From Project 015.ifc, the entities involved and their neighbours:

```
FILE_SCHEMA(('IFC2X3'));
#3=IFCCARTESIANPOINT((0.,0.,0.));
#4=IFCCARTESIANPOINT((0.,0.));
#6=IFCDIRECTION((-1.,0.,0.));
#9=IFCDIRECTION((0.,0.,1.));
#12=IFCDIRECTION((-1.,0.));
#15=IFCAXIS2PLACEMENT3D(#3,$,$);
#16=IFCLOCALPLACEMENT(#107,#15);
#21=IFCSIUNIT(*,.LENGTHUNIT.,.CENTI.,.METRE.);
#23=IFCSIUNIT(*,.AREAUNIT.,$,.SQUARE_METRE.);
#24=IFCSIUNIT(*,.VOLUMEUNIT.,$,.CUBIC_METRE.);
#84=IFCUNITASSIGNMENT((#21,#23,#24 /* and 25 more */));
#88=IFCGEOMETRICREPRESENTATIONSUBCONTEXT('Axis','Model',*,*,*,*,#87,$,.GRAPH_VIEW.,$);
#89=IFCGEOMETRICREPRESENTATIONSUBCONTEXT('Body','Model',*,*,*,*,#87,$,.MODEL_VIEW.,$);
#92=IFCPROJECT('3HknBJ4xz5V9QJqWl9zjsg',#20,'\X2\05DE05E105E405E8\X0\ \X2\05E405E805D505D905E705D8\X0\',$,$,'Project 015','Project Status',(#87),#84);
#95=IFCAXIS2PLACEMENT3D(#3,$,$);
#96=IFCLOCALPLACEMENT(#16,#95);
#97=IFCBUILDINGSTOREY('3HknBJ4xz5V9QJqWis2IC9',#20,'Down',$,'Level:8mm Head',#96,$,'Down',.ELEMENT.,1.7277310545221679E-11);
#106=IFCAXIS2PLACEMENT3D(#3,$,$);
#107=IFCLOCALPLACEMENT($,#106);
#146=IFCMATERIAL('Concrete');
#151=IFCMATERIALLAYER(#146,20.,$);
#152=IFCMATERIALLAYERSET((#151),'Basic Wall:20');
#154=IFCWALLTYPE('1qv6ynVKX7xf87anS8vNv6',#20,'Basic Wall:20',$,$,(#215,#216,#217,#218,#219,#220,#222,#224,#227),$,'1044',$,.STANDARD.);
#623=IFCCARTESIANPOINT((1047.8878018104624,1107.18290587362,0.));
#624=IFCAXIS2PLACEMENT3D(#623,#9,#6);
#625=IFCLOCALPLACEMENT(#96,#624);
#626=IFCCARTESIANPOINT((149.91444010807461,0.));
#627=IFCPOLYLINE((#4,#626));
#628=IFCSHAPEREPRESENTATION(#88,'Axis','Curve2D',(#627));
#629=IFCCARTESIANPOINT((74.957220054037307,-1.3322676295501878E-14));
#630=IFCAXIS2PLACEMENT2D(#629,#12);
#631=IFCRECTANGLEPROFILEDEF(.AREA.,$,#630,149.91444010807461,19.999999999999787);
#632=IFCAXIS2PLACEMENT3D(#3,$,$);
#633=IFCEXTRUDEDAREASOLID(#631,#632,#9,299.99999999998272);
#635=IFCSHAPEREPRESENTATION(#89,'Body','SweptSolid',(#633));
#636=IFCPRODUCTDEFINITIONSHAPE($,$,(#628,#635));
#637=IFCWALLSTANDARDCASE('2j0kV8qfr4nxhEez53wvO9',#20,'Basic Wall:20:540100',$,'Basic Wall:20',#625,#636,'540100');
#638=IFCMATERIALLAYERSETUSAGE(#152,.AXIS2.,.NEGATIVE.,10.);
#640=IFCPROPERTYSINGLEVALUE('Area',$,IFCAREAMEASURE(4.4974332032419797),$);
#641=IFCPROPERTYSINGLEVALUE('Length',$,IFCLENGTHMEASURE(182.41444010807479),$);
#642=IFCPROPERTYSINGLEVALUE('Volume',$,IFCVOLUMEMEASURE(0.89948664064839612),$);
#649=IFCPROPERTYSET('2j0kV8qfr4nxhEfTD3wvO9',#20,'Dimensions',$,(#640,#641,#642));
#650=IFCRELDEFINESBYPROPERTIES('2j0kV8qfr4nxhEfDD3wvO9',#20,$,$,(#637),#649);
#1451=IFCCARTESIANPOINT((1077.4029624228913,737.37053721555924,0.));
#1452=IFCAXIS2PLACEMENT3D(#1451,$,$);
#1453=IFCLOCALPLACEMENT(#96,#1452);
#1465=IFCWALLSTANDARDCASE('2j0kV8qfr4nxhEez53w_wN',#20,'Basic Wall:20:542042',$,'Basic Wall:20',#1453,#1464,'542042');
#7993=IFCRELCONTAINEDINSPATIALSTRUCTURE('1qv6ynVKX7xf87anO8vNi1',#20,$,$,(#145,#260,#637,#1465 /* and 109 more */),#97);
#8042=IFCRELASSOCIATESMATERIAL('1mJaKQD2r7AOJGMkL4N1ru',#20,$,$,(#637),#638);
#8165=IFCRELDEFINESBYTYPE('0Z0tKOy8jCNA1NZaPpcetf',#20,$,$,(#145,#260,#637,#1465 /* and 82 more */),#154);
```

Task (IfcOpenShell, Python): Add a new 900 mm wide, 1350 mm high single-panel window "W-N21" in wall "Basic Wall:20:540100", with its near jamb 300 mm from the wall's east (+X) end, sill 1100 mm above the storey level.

```python
import numpy as np
import ifcopenshell
import ifcopenshell.api.feature
import ifcopenshell.api.geometry
import ifcopenshell.api.pset
import ifcopenshell.api.root
import ifcopenshell.api.spatial
import ifcopenshell.api.type
import ifcopenshell.geom
import ifcopenshell.util.element
import ifcopenshell.util.placement
import ifcopenshell.util.representation
import ifcopenshell.util.shape
import ifcopenshell.util.unit

model = ifcopenshell.open("Project 015.ifc")
unit_scale = ifcopenshell.util.unit.calculate_unit_scale(model)
area_scale = ifcopenshell.util.unit.calculate_unit_scale(model, "AREAUNIT")
volume_scale = ifcopenshell.util.unit.calculate_unit_scale(model, "VOLUMEUNIT")
settings = ifcopenshell.geom.settings()


def volume(element):
    """Net volume in cubic metres, openings subtracted."""
    shape = ifcopenshell.geom.create_shape(settings, element)
    return ifcopenshell.util.shape.get_volume(shape.geometry)


wall = model.by_id(637)
storey = ifcopenshell.util.element.get_container(wall, ifc_class="IfcBuildingStorey")
context = ifcopenshell.util.representation.get_context(model, "Model", "Body", "MODEL_VIEW")
before = volume(wall)

width, height, from_end, sill = 0.9, 1.35, 0.3, 1.1  # metres

# The wall runs along its own X axis, and the end named is its -X end.
wall_shape = ifcopenshell.geom.create_shape(settings, wall)
x, y, z = ifcopenshell.util.shape.get_vertices(wall_shape.geometry).T
start = x.min() + from_end
face, thickness = float(y.min()), float(y.max() - y.min())
wall_matrix = ifcopenshell.util.placement.get_local_placement(wall.ObjectPlacement)
level = ifcopenshell.util.placement.get_local_placement(storey.ObjectPlacement)[2, 3]


def in_wall(x, y):
    """Placement at x, y metres in the wall's axes, at sill height."""
    matrix = wall_matrix.copy()
    matrix[:, 3] = wall_matrix @ np.array([x / unit_scale, y / unit_scale, 0.0, 1.0])
    matrix[2, 3] = level + sill / unit_scale
    return matrix


# Opening: a box that overshoots both wall faces by 50 mm.
opening = ifcopenshell.api.root.create_entity(model, ifc_class="IfcOpeningElement")
box = ifcopenshell.api.geometry.add_wall_representation(
    model, context=context, length=width, height=height, thickness=thickness + 0.1
)
ifcopenshell.api.geometry.assign_representation(model, product=opening, representation=box)
ifcopenshell.api.geometry.edit_object_placement(model, product=opening, matrix=in_wall(start, face - 0.05), is_si=False)
ifcopenshell.api.feature.add_feature(model, feature=opening, element=wall)

window = ifcopenshell.api.root.create_entity(model, ifc_class="IfcWindow", name="W-N21")
window.OverallWidth, window.OverallHeight = width / unit_scale, height / unit_scale
body = ifcopenshell.api.geometry.add_window_representation(
    model,
    context=context,
    overall_width=window.OverallWidth,
    overall_height=window.OverallHeight,
    partition_type="SINGLE_PANEL",
)
ifcopenshell.api.geometry.assign_representation(model, product=window, representation=body)
ifcopenshell.api.spatial.assign_container(model, products=[window], relating_structure=storey)
fills = ifcopenshell.api.feature.add_filling(model, opening=opening, element=window)
fills.OwnerHistory = window.OwnerHistory  # required in IFC2X3

# IFC2X3 keeps the operation on the window style.
style = ifcopenshell.api.root.create_entity(model, ifc_class="IfcWindowStyle", name="W-N21")
style.OperationType, style.ConstructionType = "SINGLE_PANEL", "NOTDEFINED"
style.ParameterTakesPrecedence = style.Sizeable = False
ifcopenshell.api.type.assign_type(model, related_objects=[window], relating_type=style)

# Centre the window in the wall's thickness.
ifcopenshell.api.geometry.edit_object_placement(model, product=window, matrix=in_wall(start, face), is_si=False)
window_shape = ifcopenshell.geom.create_shape(settings, window)
depth = ifcopenshell.util.shape.get_vertices(window_shape.geometry)[:, 1]
offset = face + thickness / 2 - (depth.min() + depth.max()) / 2
ifcopenshell.api.geometry.edit_object_placement(model, product=window, matrix=in_wall(start, offset), is_si=False)

after = volume(wall)

# Update the wall's stored quantities.
pset = model.by_id(ifcopenshell.util.element.get_pset(wall, "Dimensions", should_inherit=False)["id"])
ifcopenshell.api.pset.edit_pset(model, pset=pset, properties={
    "Area": model.create_entity("IfcAreaMeasure", after / thickness / area_scale),
    "Volume": model.create_entity("IfcVolumeMeasure", after / volume_scale),
})

print(f"wall volume {before:.3f} -> {after:.3f} m3")

model.write("Project 015_rev.ifc")
```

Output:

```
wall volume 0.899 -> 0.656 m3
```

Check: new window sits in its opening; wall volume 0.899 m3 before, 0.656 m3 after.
